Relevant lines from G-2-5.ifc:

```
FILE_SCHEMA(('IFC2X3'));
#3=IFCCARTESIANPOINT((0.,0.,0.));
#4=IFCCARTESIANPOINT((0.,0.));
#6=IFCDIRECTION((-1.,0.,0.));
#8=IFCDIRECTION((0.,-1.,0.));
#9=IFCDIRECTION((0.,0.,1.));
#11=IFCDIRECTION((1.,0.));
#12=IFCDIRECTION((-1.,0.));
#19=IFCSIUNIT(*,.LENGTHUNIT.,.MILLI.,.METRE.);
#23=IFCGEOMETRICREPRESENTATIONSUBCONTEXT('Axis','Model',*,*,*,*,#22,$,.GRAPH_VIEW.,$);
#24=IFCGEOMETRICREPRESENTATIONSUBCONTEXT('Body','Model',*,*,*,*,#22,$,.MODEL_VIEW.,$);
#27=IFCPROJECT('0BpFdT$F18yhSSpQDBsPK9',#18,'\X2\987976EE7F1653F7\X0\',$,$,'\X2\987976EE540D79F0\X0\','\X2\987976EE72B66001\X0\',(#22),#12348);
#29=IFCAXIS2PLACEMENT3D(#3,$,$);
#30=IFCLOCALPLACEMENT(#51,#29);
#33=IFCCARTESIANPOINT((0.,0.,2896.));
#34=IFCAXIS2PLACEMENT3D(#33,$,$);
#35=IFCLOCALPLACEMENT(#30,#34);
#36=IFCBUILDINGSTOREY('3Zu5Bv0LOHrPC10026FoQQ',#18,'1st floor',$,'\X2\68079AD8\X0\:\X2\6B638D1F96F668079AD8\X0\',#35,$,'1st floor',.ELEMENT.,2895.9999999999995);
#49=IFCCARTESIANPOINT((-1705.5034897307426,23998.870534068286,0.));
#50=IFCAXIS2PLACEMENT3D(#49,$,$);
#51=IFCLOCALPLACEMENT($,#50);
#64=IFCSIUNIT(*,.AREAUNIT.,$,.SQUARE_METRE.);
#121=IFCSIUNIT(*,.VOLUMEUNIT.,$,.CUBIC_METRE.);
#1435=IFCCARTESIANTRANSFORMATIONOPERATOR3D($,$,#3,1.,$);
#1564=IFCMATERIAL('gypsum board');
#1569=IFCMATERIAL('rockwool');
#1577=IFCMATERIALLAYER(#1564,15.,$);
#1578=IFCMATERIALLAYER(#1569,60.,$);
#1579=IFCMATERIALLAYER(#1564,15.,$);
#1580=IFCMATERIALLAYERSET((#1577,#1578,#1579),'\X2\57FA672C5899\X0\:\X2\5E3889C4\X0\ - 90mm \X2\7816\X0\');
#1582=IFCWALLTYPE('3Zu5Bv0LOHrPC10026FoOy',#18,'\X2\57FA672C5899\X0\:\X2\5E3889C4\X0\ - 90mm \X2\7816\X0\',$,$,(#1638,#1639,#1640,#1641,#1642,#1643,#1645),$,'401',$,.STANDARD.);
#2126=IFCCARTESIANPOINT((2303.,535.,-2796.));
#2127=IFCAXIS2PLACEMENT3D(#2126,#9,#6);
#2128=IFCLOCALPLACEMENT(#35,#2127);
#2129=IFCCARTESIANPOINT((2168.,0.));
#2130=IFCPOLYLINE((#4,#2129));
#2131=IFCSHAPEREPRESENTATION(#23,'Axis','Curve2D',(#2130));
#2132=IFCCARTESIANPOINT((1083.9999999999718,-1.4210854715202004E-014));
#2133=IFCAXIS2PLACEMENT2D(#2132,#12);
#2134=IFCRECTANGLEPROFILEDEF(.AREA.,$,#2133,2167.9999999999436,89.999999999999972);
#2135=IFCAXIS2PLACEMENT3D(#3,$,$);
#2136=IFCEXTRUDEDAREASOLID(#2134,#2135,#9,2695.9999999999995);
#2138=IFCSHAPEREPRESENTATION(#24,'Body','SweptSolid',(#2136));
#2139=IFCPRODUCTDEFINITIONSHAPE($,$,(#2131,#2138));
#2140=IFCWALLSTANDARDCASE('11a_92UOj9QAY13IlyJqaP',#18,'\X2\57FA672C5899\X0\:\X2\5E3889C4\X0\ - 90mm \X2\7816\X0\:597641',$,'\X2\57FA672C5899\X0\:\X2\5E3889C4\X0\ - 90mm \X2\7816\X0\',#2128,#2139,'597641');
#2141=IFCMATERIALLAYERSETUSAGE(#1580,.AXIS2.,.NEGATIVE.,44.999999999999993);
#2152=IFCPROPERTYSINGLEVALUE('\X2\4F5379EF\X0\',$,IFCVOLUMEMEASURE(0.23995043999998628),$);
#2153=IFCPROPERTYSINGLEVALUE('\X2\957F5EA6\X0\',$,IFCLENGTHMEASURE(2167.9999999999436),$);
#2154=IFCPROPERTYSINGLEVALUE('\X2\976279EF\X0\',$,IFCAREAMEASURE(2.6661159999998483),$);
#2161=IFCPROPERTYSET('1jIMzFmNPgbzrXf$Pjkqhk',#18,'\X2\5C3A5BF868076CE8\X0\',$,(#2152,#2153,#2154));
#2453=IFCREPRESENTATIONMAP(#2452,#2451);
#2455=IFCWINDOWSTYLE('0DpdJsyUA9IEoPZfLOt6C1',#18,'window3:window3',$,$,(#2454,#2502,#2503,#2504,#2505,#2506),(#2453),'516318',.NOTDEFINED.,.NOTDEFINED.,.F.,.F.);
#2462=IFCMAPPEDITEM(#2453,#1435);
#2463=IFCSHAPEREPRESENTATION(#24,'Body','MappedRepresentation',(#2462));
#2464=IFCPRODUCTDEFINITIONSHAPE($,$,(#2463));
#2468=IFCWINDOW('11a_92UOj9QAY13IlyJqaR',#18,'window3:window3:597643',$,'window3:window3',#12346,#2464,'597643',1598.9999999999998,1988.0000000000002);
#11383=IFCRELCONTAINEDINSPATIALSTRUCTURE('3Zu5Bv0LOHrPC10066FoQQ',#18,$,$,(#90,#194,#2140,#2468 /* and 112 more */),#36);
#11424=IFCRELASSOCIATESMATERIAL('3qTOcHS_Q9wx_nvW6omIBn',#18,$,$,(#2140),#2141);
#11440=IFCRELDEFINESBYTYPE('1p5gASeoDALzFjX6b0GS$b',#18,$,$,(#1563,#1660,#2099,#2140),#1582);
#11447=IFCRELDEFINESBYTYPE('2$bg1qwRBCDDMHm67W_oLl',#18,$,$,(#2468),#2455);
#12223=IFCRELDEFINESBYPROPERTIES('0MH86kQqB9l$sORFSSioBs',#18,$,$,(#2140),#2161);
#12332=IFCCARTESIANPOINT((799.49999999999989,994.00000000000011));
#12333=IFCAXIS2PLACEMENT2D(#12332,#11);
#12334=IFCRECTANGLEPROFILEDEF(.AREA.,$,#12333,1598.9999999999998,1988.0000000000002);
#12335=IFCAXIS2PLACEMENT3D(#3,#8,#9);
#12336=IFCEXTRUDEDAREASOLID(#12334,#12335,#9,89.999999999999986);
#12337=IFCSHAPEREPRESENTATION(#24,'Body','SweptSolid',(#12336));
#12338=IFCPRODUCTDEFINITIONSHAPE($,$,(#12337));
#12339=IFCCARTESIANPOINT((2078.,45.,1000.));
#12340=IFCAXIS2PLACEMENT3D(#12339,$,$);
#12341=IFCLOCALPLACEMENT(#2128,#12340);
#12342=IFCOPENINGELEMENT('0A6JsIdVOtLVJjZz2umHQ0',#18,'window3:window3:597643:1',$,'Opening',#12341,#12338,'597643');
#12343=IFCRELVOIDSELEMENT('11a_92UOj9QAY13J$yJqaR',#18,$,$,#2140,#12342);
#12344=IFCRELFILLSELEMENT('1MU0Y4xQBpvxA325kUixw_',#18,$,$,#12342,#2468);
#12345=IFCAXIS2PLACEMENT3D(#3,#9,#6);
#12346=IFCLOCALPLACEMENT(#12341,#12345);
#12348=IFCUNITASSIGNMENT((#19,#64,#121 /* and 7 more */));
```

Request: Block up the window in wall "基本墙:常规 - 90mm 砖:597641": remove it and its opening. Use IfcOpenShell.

```python
import ifcopenshell
import ifcopenshell.api.feature
import ifcopenshell.api.pset
import ifcopenshell.api.root
import ifcopenshell.geom
import ifcopenshell.util.element
import ifcopenshell.util.shape
import ifcopenshell.util.unit

model = ifcopenshell.open("G-2-5.ifc")
area_scale = ifcopenshell.util.unit.calculate_unit_scale(model, "AREAUNIT")
volume_scale = ifcopenshell.util.unit.calculate_unit_scale(model, "VOLUMEUNIT")
settings = ifcopenshell.geom.settings()


def volume(element):
    """Net volume in cubic metres, openings subtracted."""
    shape = ifcopenshell.geom.create_shape(settings, element)
    return ifcopenshell.util.shape.get_volume(shape.geometry)


window = model.by_id(2468)
opening = window.FillsVoids[0].RelatingOpeningElement
wall = opening.VoidsElements[0].RelatingBuildingElement
before = volume(wall)

ifcopenshell.api.root.remove_product(model, product=window)
ifcopenshell.api.feature.remove_feature(model, feature=opening)

after = volume(wall)
thickness = 0.09  # wall thickness in metres

# Update the wall's stored quantities.
pset = model.by_id(ifcopenshell.util.element.get_pset(wall, "尺寸标注", should_inherit=False)["id"])
ifcopenshell.api.pset.edit_pset(model, pset=pset, properties={
    "体积": model.create_entity("IfcVolumeMeasure", after / volume_scale),
    "面积": model.create_entity("IfcAreaMeasure", after / thickness / area_scale),
})

print(f"wall volume {before:.3f} -> {after:.3f} m3")

model.write("G-2-5_edited.ifc")
```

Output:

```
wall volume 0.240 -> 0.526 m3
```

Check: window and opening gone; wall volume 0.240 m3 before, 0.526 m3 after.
